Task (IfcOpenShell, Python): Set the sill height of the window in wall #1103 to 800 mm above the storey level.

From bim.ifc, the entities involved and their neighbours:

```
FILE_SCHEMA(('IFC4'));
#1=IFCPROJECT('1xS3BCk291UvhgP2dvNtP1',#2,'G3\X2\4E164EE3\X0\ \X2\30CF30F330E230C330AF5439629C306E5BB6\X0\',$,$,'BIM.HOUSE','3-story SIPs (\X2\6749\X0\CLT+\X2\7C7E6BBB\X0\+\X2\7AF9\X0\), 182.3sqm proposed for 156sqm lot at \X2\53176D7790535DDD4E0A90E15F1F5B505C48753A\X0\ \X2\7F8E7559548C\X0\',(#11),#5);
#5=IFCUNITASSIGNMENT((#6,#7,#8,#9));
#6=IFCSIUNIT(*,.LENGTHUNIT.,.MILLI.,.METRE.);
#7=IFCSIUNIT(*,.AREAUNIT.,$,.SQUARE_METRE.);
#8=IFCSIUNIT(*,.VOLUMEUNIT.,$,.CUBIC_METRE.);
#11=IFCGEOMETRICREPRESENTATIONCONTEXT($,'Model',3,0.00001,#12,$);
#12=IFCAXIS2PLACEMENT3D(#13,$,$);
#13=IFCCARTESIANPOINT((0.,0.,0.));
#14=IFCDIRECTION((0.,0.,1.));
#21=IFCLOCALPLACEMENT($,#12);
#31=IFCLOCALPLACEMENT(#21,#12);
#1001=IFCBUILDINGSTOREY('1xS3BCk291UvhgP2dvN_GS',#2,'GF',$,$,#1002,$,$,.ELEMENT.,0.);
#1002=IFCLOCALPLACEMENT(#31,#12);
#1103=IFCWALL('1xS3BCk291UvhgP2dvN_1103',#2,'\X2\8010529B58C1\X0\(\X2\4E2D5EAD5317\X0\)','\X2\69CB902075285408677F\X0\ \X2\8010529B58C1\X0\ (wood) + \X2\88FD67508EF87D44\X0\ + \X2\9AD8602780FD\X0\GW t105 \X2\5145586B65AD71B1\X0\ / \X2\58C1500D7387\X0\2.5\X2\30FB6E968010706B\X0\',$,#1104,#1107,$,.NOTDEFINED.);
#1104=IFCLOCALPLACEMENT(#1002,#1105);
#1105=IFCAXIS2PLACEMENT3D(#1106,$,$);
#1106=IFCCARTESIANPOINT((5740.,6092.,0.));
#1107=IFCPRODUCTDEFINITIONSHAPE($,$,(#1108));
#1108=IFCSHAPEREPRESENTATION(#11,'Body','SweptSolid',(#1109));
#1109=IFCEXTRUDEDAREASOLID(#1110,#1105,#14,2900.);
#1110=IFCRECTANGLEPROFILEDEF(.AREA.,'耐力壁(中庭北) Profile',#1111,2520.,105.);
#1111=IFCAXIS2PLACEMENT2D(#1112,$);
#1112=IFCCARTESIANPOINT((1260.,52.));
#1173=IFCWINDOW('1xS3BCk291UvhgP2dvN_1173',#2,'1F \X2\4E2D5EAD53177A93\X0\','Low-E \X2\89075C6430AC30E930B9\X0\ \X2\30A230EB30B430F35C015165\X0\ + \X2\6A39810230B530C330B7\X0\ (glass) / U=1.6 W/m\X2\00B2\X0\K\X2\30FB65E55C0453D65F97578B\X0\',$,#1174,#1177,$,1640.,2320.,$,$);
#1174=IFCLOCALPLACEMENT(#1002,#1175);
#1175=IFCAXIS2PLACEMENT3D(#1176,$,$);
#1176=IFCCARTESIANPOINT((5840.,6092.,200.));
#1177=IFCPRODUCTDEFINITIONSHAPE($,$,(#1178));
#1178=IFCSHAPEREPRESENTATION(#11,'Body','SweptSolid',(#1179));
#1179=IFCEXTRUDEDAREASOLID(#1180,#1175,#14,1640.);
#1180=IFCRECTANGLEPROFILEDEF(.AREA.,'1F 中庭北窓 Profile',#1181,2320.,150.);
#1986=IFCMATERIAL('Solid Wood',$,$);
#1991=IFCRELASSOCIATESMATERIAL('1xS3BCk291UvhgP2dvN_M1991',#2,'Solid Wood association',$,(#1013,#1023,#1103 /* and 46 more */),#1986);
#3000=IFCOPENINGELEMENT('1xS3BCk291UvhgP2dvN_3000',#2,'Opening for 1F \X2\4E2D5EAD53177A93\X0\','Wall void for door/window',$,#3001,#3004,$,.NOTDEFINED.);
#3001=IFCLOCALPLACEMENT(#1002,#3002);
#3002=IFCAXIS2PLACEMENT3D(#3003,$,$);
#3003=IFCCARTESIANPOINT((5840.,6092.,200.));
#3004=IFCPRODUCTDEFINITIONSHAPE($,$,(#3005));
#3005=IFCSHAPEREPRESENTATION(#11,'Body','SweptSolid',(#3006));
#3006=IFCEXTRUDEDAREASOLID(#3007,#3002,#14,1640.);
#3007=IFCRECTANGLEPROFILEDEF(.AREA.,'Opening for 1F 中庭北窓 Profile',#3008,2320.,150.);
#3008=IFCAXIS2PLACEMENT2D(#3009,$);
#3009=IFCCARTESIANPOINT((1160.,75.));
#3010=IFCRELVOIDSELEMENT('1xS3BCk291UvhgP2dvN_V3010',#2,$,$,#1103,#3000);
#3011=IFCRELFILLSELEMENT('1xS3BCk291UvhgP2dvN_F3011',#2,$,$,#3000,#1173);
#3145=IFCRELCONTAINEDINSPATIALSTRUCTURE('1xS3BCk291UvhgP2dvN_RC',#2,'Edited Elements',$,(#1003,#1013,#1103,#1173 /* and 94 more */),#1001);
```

```python
import numpy as np
import ifcopenshell
import ifcopenshell.api.geometry
import ifcopenshell.geom
import ifcopenshell.util.element
import ifcopenshell.util.placement
import ifcopenshell.util.shape
import ifcopenshell.util.unit

model = ifcopenshell.open("bim.ifc")
unit_scale = ifcopenshell.util.unit.calculate_unit_scale(model)

window = model.by_guid("1xS3BCk291UvhgP2dvN_1173")
opening = window.FillsVoids[0].RelatingOpeningElement
storey = ifcopenshell.util.element.get_container(window, ifc_class="IfcBuildingStorey")
level = ifcopenshell.util.placement.get_local_placement(storey.ObjectPlacement)[2, 3]

# The opening's origin need not be at the sill, so measure its lowest point.
shape = ifcopenshell.geom.create_shape(ifcopenshell.geom.settings(), opening)
bottom = ifcopenshell.util.shape.get_shape_bottom_elevation(shape, shape.geometry) / unit_scale
dz = level + 0.8 / unit_scale - bottom

shift = np.array([0.0, 0.0, dz])
# The window is not placed relative to its opening, so move both.
for product in (opening, window):
    matrix = ifcopenshell.util.placement.get_local_placement(product.ObjectPlacement)
    matrix[:3, 3] += shift
    ifcopenshell.api.geometry.edit_object_placement(model, product=product, matrix=matrix, is_si=False)

print(f"moved by {dz * unit_scale:+.3f} m")

model.write("bim_rev.ifc")
```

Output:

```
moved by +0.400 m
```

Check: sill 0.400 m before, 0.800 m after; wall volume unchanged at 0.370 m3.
